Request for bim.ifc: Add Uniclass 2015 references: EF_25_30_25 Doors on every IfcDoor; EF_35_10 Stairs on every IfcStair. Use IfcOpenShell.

First a look at what the model holds.

```python
import ifcopenshell

model = ifcopenshell.open("bim.ifc")
print(model.schema)
print("classifications:", [c.Name for c in model.by_type("IfcClassification")])
for ifc_class in ("IfcDoor", "IfcRoof", "IfcStair", "IfcWall", "IfcWindow"):
    print(ifc_class, len(model.by_type(ifc_class)))
```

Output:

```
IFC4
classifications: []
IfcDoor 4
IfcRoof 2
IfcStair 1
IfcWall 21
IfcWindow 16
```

```python
import ifcopenshell
import ifcopenshell.api.classification

model = ifcopenshell.open("bim.ifc")

system = ifcopenshell.api.classification.add_classification(model, classification="Uniclass 2015")

codes = {
    "IfcDoor": ("EF_25_30_25", "Doors"),
    "IfcStair": ("EF_35_10", "Stairs"),
}
for ifc_class, (code, name) in codes.items():
    products = model.by_type(ifc_class)
    ifcopenshell.api.classification.add_reference(
        model, products=products, classification=system, identification=code, name=name
    )
    print(code, len(products))

model.write("bim_rev.ifc")
```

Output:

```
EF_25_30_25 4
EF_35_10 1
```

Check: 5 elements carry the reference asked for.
